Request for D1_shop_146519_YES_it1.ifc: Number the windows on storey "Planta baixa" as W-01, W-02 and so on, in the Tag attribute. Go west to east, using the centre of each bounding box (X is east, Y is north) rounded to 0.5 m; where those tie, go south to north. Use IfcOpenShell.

First a look at what the model holds.

```python
import ifcopenshell
import ifcopenshell.util.element
import ifcopenshell.util.placement

model = ifcopenshell.open("D1_shop_146519_YES_it1.ifc")
print(model.schema)
storey = next(s for s in model.by_type("IfcBuildingStorey") if s.Name == "Planta baixa")
windows = [e for e in ifcopenshell.util.element.get_decomposition(storey) if e.is_a("IfcWindow")]
for e in sorted(windows, key=lambda e: e.id()):
    origin = ifcopenshell.util.placement.get_local_placement(e.ObjectPlacement)[:3, 3]
    print(e.id(), e.Tag, e.Name, origin.round(2) + 0.0, sep=" | ")
```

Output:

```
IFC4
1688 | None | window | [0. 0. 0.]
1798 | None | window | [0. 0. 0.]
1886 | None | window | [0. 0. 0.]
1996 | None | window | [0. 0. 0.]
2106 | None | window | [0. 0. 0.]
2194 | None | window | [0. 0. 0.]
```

```python
import ifcopenshell
import ifcopenshell.geom
import ifcopenshell.util.element
import ifcopenshell.util.shape

model = ifcopenshell.open("D1_shop_146519_YES_it1.ifc")
settings = ifcopenshell.geom.settings()
settings.set("use-world-coords", True)


def centre(element):
    shape = ifcopenshell.geom.create_shape(settings, element)
    return ifcopenshell.util.shape.get_bbox_centroid(shape.geometry)


storey = next(s for s in model.by_type("IfcBuildingStorey") if s.Name == "Planta baixa")
windows = [e for e in ifcopenshell.util.element.get_decomposition(storey) if e.is_a("IfcWindow")]

# Insertion points can sit at a corner or the storey origin, so sort by the geometry (in metres).
centres = {e: centre(e) for e in windows}
windows.sort(key=lambda e: (round(centres[e][0] / 0.5), centres[e][1]))

for i, e in enumerate(windows, start=1):
    number = f"W-{i:02d}"
    e.Tag = number
    print(e.id(), number)

model.write("D1_shop_146519_YES_it1_v2.ifc")
```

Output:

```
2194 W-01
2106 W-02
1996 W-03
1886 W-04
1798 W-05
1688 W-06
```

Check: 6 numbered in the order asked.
